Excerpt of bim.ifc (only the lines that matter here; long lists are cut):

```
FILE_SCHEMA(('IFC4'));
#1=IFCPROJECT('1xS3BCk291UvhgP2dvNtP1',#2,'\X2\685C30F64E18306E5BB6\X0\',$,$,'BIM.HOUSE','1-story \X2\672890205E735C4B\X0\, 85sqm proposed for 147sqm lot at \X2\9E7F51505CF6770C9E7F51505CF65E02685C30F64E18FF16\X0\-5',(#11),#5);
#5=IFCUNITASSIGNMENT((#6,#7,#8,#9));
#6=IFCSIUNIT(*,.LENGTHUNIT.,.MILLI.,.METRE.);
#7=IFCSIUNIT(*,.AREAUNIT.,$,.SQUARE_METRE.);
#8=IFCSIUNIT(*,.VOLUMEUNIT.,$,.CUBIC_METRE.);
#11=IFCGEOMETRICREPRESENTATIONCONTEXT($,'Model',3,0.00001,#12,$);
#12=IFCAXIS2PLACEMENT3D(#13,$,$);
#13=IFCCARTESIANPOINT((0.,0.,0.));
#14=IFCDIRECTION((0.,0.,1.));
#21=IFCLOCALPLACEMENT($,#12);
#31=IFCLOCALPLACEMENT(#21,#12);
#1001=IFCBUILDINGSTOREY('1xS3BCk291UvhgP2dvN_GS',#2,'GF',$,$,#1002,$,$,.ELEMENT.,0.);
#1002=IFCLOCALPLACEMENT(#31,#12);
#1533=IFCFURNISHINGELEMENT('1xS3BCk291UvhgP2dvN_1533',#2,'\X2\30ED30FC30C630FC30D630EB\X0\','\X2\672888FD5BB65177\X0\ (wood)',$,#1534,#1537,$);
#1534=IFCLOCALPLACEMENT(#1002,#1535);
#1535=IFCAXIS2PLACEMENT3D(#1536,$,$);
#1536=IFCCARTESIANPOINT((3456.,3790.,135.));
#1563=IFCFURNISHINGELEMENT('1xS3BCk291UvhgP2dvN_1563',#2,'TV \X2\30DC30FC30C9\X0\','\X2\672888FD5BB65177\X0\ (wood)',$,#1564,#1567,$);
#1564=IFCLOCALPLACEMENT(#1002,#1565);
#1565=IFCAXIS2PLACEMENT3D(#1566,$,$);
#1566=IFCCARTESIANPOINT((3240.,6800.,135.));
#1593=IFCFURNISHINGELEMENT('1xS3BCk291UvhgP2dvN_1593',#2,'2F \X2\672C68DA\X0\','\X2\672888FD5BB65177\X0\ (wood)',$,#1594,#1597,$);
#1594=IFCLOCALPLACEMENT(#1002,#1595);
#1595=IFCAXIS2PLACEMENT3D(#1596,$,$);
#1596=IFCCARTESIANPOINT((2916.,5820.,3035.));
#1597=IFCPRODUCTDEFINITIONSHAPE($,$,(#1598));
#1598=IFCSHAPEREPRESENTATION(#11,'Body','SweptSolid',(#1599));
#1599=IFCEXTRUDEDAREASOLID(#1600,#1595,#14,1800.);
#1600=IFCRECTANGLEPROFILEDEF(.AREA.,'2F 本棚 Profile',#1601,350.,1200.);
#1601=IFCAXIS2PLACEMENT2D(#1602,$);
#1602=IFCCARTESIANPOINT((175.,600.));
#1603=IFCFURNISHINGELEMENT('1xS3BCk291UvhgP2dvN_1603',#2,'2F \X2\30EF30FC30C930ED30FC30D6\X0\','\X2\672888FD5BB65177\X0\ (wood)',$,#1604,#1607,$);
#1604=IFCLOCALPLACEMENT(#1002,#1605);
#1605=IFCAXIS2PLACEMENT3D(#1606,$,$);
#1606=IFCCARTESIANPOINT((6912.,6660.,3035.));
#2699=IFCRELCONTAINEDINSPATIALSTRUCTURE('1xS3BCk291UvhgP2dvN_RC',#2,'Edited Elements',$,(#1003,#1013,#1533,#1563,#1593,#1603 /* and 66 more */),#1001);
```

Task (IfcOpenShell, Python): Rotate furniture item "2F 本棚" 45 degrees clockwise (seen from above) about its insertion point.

```python
import ifcopenshell
import ifcopenshell.api.geometry
import ifcopenshell.util.placement

model = ifcopenshell.open("bim.ifc")

item = model.by_guid("1xS3BCk291UvhgP2dvN_1593")
matrix = ifcopenshell.util.placement.get_local_placement(item.ObjectPlacement)
matrix = matrix @ ifcopenshell.util.placement.rotation(-45, "Z")
ifcopenshell.api.geometry.edit_object_placement(model, product=item, matrix=matrix, is_si=False)

print(ifcopenshell.util.placement.get_local_placement(item.ObjectPlacement).round(3) + 0.0)

model.write("bim_rev.ifc")
```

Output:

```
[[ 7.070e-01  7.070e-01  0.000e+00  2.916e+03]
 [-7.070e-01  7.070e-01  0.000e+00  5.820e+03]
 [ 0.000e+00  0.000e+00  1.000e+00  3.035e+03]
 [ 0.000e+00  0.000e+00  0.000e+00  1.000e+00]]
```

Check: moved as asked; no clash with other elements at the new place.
